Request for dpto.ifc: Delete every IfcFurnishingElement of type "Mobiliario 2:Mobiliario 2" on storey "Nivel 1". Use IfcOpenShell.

First a look at what the model holds.

```python
import ifcopenshell
import ifcopenshell.util.element

model = ifcopenshell.open("dpto.ifc")
print(model.schema)
storey = next(s for s in model.by_type("IfcBuildingStorey") if s.Name == "Nivel 1")
furniture = [e for e in ifcopenshell.util.element.get_decomposition(storey) if e.is_a("IfcFurnishingElement")]
seen = {}
for e in furniture:
    element_type = ifcopenshell.util.element.get_type(e)
    name = element_type.Name if element_type not in (None, e) else None
    seen[name] = seen.get(name, 0) + 1
for name, count in sorted(seen.items(), key=str):
    print(count, "x", name)
```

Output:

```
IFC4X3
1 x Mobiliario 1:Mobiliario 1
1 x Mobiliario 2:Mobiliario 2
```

```python
import ifcopenshell
import ifcopenshell.api.root
import ifcopenshell.util.element

model = ifcopenshell.open("dpto.ifc")

storey = next(s for s in model.by_type("IfcBuildingStorey") if s.Name == "Nivel 1")
furniture = [e for e in ifcopenshell.util.element.get_decomposition(storey) if e.is_a("IfcFurnishingElement")]
targets = [e for e in furniture if (t := ifcopenshell.util.element.get_type(e)) not in (None, e) and t.Name == "Mobiliario 2:Mobiliario 2"]

for e in targets:
    ifcopenshell.api.root.remove_product(model, product=e)
print(len(targets), "removed")

model.write("dpto-out.ifc")
```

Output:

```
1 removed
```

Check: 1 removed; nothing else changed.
